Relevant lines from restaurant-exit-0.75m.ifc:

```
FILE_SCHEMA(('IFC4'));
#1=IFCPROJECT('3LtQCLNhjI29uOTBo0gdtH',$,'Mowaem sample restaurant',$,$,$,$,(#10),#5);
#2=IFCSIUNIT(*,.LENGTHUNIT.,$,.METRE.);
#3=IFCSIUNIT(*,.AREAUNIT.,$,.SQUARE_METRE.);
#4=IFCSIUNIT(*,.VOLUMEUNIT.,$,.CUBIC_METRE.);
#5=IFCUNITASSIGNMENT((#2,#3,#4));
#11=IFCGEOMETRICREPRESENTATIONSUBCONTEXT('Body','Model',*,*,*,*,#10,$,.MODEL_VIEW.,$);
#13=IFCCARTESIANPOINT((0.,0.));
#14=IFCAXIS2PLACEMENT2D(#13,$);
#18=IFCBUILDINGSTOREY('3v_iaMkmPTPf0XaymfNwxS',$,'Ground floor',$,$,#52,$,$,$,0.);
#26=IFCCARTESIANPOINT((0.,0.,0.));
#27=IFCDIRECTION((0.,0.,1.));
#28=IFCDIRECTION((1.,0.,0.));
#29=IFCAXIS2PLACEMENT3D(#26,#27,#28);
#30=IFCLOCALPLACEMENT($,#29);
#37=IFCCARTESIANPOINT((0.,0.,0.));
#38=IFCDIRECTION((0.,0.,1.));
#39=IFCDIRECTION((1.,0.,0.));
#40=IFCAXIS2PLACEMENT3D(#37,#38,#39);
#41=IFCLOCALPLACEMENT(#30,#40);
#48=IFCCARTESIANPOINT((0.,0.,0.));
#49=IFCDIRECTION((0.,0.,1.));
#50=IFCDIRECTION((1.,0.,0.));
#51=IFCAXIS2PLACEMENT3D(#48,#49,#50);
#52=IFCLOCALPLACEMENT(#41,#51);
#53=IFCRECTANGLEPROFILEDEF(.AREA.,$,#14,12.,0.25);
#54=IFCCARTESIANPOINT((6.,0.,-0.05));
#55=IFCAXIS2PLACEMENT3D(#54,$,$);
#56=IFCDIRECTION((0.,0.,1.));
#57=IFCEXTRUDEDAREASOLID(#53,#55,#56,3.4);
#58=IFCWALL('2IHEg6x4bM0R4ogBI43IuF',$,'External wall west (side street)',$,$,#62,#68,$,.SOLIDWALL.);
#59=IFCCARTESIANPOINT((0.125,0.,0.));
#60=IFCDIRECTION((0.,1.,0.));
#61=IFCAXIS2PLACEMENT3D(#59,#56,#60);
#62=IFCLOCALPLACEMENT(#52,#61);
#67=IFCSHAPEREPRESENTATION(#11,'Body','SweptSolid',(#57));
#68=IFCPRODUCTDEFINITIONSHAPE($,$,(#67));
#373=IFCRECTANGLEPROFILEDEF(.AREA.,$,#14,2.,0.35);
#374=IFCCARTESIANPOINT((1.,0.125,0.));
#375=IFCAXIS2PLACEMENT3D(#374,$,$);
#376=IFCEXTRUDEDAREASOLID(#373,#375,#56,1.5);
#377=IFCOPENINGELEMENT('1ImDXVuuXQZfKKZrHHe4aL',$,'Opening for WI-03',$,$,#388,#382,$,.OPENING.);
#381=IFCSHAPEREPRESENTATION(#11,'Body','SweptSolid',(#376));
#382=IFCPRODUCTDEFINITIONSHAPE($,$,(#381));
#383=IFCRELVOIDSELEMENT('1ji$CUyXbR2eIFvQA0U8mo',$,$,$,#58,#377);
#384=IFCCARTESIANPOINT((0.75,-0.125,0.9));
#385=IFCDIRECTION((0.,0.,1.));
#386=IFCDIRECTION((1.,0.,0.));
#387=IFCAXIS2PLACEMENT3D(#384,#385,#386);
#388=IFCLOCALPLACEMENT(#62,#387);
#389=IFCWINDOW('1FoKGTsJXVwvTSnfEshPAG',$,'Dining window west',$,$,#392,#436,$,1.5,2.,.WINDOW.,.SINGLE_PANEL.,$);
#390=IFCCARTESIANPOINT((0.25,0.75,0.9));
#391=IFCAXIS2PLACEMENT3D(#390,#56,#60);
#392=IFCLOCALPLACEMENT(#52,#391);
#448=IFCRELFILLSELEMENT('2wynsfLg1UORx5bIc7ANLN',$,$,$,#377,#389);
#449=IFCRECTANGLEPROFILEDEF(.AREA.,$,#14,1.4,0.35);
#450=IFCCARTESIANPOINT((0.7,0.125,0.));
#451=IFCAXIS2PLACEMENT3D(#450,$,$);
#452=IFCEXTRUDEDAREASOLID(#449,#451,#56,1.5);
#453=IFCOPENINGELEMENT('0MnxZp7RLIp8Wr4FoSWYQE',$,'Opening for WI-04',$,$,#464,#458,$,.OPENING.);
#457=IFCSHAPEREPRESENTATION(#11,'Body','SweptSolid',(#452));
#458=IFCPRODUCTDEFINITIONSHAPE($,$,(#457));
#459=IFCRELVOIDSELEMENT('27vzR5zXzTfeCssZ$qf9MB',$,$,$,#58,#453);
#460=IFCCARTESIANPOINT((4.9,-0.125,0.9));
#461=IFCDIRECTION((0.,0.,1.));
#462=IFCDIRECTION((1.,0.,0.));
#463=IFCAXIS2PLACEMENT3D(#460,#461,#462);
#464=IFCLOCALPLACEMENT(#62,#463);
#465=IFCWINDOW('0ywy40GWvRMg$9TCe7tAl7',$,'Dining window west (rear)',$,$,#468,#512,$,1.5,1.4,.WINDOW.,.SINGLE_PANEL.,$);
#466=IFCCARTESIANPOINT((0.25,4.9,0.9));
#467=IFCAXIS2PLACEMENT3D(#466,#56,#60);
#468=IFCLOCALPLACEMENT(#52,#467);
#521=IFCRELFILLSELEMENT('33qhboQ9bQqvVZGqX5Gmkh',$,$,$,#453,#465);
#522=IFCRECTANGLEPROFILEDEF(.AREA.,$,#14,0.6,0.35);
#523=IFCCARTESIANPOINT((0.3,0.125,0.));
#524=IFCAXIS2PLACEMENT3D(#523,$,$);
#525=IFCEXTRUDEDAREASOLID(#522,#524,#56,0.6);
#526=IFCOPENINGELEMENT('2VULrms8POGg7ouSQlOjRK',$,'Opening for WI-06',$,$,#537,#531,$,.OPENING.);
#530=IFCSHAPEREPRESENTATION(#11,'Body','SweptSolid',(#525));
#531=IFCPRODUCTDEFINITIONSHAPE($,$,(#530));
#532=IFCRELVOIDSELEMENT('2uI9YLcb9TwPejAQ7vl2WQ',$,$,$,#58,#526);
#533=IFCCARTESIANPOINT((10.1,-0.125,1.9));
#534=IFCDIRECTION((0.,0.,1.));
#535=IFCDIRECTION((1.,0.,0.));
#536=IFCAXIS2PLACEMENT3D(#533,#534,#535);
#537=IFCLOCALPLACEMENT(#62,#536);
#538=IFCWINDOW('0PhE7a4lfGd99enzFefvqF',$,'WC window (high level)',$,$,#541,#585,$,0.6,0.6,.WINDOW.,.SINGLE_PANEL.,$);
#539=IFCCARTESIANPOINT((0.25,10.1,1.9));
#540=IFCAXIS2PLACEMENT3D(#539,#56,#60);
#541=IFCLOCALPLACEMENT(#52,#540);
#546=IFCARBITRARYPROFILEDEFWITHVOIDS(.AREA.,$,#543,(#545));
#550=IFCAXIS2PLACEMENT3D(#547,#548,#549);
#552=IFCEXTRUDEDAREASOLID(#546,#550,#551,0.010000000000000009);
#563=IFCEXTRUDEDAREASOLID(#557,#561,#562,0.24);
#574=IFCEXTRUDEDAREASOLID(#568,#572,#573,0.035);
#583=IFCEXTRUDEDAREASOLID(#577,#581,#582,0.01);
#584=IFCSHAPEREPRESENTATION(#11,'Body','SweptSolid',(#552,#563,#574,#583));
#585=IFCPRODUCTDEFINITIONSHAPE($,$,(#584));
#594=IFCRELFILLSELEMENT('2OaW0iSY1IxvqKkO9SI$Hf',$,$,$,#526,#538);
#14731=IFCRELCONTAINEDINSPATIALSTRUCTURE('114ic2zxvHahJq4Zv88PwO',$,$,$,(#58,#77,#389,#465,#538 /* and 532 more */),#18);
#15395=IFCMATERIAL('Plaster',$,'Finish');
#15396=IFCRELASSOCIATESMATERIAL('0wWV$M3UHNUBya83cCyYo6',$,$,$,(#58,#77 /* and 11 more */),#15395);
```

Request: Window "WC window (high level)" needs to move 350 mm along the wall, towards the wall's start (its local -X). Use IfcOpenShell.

```python
import ifcopenshell
import ifcopenshell.api.geometry
import ifcopenshell.util.placement

model = ifcopenshell.open("restaurant-exit-0.75m.ifc")

window = model.by_guid("0PhE7a4lfGd99enzFefvqF")
opening = window.FillsVoids[0].RelatingOpeningElement
wall = opening.VoidsElements[0].RelatingBuildingElement

wall_matrix = ifcopenshell.util.placement.get_local_placement(wall.ObjectPlacement)
shift = wall_matrix[:3, 0] * -0.35
before = ifcopenshell.util.placement.get_local_placement(window.ObjectPlacement)[:3, 3].copy()

# The window is not placed relative to its opening, so move both.
for product in (opening, window):
    matrix = ifcopenshell.util.placement.get_local_placement(product.ObjectPlacement)
    matrix[:3, 3] += shift
    ifcopenshell.api.geometry.edit_object_placement(model, product=product, matrix=matrix, is_si=False)

after = ifcopenshell.util.placement.get_local_placement(window.ObjectPlacement)[:3, 3]
print("window moved by", (after - before).round(3) + 0.0)

model.write("restaurant-exit-0.75m_updated.ifc")
```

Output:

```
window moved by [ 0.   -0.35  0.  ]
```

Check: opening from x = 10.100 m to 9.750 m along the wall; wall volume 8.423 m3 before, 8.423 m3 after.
